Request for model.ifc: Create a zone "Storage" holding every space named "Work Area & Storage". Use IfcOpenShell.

First a look at what the model holds.

```python
import ifcopenshell

model = ifcopenshell.open("model.ifc")
print(model.schema)
seen = {}
for space in model.by_type("IfcSpace"):
    seen[space.LongName] = seen.get(space.LongName, 0) + 1
for name, count in sorted(seen.items(), key=str):
    print(count, "x", name)
print("zones:", [z.Name for z in model.by_type("IfcZone")][:20])
```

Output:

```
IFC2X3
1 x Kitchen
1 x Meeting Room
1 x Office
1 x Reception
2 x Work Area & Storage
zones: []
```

```python
import ifcopenshell
import ifcopenshell.api.group
import ifcopenshell.api.root

model = ifcopenshell.open("model.ifc")

names = {"Work Area & Storage"}
spaces = [s for s in model.by_type("IfcSpace") if s.LongName in names]

zone = ifcopenshell.api.root.create_entity(model, ifc_class="IfcZone", name="Storage")
ifcopenshell.api.group.assign_group(model, products=spaces, group=zone)
print(len(spaces), "spaces in", zone.Name)

model.write("model_rev.ifc")
```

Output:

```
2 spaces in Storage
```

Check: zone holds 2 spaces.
